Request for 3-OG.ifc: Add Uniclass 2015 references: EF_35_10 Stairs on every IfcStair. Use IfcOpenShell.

First a look at what the model holds.

```python
import ifcopenshell

model = ifcopenshell.open("3-OG.ifc")
print(model.schema)
print("classifications:", [c.Name for c in model.by_type("IfcClassification")])
for ifc_class in ("IfcDoor", "IfcRoof", "IfcStair", "IfcWall", "IfcWindow"):
    print(ifc_class, len(model.by_type(ifc_class)))
```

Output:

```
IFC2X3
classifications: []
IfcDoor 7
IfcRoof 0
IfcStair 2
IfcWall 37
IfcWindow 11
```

```python
import ifcopenshell
import ifcopenshell.api.classification

model = ifcopenshell.open("3-OG.ifc")

# IFC2X3 requires Source and Edition and has no link from the project to the system.
system = model.create_entity("IfcClassification", Source="NBS", Edition="2015", Name="Uniclass 2015")

codes = {
    "IfcStair": ("EF_35_10", "Stairs"),
}
for ifc_class, (code, name) in codes.items():
    products = model.by_type(ifc_class)
    ifcopenshell.api.classification.add_reference(
        model, products=products, classification=system, identification=code, name=name
    )
    print(code, len(products))

model.write("3-OG-out.ifc")
```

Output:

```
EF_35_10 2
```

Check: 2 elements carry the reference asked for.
